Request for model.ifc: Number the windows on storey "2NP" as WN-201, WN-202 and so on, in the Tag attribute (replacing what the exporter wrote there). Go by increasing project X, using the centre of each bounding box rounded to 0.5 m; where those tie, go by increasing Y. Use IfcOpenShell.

First a look at what the model holds.

```python
import ifcopenshell
import ifcopenshell.util.element
import ifcopenshell.util.placement

model = ifcopenshell.open("model.ifc")
print(model.schema)
storey = next(s for s in model.by_type("IfcBuildingStorey") if s.Name == "2NP")
windows = [e for e in ifcopenshell.util.element.get_decomposition(storey) if e.is_a("IfcWindow")]
for e in sorted(windows, key=lambda e: e.id()):
    origin = ifcopenshell.util.placement.get_local_placement(e.ObjectPlacement)[:3, 3]
    print(e.id(), e.Tag, e.Name, origin.round(2) + 0.0, sep=" | ")
```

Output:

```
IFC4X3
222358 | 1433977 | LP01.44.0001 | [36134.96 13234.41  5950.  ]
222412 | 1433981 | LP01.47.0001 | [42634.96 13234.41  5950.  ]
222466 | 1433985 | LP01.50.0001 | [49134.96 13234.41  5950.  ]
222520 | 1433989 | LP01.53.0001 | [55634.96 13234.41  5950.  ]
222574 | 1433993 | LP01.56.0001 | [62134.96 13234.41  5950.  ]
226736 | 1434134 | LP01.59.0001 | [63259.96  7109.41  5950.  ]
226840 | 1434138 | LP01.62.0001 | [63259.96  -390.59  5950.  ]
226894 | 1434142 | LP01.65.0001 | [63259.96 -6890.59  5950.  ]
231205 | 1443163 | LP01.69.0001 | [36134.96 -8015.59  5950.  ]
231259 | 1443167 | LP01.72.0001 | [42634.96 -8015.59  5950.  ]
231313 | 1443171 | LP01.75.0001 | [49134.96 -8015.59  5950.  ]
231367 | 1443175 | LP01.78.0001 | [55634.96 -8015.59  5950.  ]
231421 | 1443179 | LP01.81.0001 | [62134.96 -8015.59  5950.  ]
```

```python
import ifcopenshell
import ifcopenshell.geom
import ifcopenshell.util.element
import ifcopenshell.util.shape

model = ifcopenshell.open("model.ifc")
settings = ifcopenshell.geom.settings()
settings.set("use-world-coords", True)


def centre(element):
    shape = ifcopenshell.geom.create_shape(settings, element)
    return ifcopenshell.util.shape.get_bbox_centroid(shape.geometry)


storey = next(s for s in model.by_type("IfcBuildingStorey") if s.Name == "2NP")
windows = [e for e in ifcopenshell.util.element.get_decomposition(storey) if e.is_a("IfcWindow")]

# Insertion points can sit at a corner or the storey origin, so sort by the geometry (in metres).
centres = {e: centre(e) for e in windows}
windows.sort(key=lambda e: (round(centres[e][0] / 0.5), centres[e][1]))

for i, e in enumerate(windows, start=1):
    number = f"WN-2{i:02d}"
    e.Tag = number
    print(e.id(), number)

model.write("model_v2.ifc")
```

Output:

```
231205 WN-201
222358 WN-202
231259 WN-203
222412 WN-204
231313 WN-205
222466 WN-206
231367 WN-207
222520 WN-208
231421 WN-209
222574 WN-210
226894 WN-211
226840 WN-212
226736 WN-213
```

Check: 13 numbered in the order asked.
